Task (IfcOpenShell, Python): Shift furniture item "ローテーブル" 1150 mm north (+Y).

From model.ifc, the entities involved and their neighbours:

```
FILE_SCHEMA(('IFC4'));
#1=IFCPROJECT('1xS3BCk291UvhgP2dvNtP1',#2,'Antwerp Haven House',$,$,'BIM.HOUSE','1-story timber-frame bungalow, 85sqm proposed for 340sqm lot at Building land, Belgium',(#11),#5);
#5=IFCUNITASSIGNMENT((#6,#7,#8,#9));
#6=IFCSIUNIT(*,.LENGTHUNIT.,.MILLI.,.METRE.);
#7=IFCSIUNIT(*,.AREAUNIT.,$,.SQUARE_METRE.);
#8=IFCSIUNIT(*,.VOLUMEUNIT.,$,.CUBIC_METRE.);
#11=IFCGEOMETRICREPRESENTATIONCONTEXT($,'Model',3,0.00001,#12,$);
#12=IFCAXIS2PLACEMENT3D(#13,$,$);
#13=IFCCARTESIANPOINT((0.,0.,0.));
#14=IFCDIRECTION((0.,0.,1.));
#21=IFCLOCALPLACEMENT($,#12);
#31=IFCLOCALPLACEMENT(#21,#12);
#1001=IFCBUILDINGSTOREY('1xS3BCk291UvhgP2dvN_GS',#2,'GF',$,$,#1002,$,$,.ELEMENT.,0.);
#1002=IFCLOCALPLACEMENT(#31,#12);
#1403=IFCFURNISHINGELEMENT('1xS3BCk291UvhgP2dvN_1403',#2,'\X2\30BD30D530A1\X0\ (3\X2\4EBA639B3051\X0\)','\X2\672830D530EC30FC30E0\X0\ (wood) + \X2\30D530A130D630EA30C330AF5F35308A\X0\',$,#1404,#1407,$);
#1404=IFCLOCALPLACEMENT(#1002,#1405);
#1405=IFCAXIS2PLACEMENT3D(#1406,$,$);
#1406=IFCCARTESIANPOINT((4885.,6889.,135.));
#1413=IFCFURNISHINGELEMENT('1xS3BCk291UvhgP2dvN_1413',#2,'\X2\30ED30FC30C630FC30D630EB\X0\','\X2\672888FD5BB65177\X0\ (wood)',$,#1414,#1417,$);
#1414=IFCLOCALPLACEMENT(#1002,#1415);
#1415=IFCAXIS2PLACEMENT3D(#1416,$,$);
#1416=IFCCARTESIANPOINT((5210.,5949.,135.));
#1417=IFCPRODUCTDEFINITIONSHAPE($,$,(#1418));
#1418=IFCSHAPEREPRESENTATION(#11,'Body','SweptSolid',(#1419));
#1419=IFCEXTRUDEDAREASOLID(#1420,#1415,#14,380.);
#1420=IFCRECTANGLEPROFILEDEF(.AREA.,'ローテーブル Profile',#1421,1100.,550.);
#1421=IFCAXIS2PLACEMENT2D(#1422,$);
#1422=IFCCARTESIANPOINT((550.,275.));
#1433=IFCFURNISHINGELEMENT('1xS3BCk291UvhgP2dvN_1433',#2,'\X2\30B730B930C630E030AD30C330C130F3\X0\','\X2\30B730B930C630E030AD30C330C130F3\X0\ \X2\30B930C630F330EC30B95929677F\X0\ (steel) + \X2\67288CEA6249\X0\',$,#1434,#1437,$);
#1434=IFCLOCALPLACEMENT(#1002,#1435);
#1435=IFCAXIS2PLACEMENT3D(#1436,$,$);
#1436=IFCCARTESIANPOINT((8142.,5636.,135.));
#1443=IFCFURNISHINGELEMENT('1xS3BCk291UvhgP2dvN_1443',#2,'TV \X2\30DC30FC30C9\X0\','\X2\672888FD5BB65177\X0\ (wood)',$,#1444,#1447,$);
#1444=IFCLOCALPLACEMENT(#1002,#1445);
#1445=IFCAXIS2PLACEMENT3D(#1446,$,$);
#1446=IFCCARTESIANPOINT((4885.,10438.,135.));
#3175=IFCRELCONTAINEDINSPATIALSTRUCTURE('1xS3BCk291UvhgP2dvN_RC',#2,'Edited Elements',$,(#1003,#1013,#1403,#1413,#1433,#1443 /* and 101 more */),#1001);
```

```python
import ifcopenshell
import ifcopenshell.api.geometry
import ifcopenshell.util.placement
import ifcopenshell.util.unit

model = ifcopenshell.open("model.ifc")
unit_scale = ifcopenshell.util.unit.calculate_unit_scale(model)

item = model.by_guid("1xS3BCk291UvhgP2dvN_1413")
matrix = ifcopenshell.util.placement.get_local_placement(item.ObjectPlacement)
matrix[1, 3] += 1.15 / unit_scale
ifcopenshell.api.geometry.edit_object_placement(model, product=item, matrix=matrix, is_si=False)

print(ifcopenshell.util.placement.get_local_placement(item.ObjectPlacement).round(3) + 0.0)

model.write("model_updated.ifc")
```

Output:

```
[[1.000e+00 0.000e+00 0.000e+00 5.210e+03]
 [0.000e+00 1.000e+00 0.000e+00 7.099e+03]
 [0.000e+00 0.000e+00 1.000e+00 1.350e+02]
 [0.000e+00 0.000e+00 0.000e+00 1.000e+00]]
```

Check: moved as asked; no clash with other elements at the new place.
